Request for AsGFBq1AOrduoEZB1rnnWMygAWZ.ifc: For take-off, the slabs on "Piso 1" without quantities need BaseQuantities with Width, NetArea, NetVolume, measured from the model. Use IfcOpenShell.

First a look at what the model holds.

```python
import ifcopenshell
import ifcopenshell.util.element
import ifcopenshell.util.unit

model = ifcopenshell.open("AsGFBq1AOrduoEZB1rnnWMygAWZ.ifc")
print(model.schema)
for unit_type in ("LENGTHUNIT", "AREAUNIT", "VOLUMEUNIT"):
    print(unit_type, ifcopenshell.util.unit.calculate_unit_scale(model, unit_type))
storey = next(s for s in model.by_type("IfcBuildingStorey") if s.Name == "Piso 1")
slabs = [e for e in ifcopenshell.util.element.get_decomposition(storey) if e.is_a("IfcSlab")]
for e in sorted(slabs, key=lambda e: e.id()):
    print(e.id(), e.is_a(), e.Name, list(ifcopenshell.util.element.get_psets(e, qtos_only=True)), sep=" | ")
```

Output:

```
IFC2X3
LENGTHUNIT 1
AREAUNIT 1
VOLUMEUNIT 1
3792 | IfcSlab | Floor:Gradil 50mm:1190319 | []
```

```python
import ifcopenshell
import ifcopenshell.api.pset
import ifcopenshell.geom
import ifcopenshell.util.element
import ifcopenshell.util.shape
import ifcopenshell.util.unit

model = ifcopenshell.open("AsGFBq1AOrduoEZB1rnnWMygAWZ.ifc")
unit_scale = ifcopenshell.util.unit.calculate_unit_scale(model)
area_scale = ifcopenshell.util.unit.calculate_unit_scale(model, "AREAUNIT")
volume_scale = ifcopenshell.util.unit.calculate_unit_scale(model, "VOLUMEUNIT")
settings = ifcopenshell.geom.settings()

storey = next(s for s in model.by_type("IfcBuildingStorey") if s.Name == "Piso 1")
slabs = [e for e in ifcopenshell.util.element.get_decomposition(storey) if e.is_a("IfcSlab")]

for e in sorted(slabs, key=lambda e: e.id()):
    if ifcopenshell.util.element.get_psets(e, qtos_only=True, should_inherit=False):
        continue
    # Geometry comes back in metres, in the element's own axes.
    shape = ifcopenshell.geom.create_shape(settings, e)
    values = {
        "Width": ifcopenshell.util.shape.get_z(shape.geometry) / unit_scale,
        "NetArea": ifcopenshell.util.shape.get_footprint_area(shape.geometry) / area_scale,
        "NetVolume": ifcopenshell.util.shape.get_volume(shape.geometry) / volume_scale,
    }
    qto = ifcopenshell.api.pset.add_qto(model, product=e, name="BaseQuantities")
    ifcopenshell.api.pset.edit_qto(model, qto=qto, properties=values)
    print(e.id(), {k: round(v, 3) for k, v in values.items()})

model.write("AsGFBq1AOrduoEZB1rnnWMygAWZ_edited.ifc")
```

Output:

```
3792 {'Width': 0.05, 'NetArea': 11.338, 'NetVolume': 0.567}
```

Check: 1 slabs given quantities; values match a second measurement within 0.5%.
